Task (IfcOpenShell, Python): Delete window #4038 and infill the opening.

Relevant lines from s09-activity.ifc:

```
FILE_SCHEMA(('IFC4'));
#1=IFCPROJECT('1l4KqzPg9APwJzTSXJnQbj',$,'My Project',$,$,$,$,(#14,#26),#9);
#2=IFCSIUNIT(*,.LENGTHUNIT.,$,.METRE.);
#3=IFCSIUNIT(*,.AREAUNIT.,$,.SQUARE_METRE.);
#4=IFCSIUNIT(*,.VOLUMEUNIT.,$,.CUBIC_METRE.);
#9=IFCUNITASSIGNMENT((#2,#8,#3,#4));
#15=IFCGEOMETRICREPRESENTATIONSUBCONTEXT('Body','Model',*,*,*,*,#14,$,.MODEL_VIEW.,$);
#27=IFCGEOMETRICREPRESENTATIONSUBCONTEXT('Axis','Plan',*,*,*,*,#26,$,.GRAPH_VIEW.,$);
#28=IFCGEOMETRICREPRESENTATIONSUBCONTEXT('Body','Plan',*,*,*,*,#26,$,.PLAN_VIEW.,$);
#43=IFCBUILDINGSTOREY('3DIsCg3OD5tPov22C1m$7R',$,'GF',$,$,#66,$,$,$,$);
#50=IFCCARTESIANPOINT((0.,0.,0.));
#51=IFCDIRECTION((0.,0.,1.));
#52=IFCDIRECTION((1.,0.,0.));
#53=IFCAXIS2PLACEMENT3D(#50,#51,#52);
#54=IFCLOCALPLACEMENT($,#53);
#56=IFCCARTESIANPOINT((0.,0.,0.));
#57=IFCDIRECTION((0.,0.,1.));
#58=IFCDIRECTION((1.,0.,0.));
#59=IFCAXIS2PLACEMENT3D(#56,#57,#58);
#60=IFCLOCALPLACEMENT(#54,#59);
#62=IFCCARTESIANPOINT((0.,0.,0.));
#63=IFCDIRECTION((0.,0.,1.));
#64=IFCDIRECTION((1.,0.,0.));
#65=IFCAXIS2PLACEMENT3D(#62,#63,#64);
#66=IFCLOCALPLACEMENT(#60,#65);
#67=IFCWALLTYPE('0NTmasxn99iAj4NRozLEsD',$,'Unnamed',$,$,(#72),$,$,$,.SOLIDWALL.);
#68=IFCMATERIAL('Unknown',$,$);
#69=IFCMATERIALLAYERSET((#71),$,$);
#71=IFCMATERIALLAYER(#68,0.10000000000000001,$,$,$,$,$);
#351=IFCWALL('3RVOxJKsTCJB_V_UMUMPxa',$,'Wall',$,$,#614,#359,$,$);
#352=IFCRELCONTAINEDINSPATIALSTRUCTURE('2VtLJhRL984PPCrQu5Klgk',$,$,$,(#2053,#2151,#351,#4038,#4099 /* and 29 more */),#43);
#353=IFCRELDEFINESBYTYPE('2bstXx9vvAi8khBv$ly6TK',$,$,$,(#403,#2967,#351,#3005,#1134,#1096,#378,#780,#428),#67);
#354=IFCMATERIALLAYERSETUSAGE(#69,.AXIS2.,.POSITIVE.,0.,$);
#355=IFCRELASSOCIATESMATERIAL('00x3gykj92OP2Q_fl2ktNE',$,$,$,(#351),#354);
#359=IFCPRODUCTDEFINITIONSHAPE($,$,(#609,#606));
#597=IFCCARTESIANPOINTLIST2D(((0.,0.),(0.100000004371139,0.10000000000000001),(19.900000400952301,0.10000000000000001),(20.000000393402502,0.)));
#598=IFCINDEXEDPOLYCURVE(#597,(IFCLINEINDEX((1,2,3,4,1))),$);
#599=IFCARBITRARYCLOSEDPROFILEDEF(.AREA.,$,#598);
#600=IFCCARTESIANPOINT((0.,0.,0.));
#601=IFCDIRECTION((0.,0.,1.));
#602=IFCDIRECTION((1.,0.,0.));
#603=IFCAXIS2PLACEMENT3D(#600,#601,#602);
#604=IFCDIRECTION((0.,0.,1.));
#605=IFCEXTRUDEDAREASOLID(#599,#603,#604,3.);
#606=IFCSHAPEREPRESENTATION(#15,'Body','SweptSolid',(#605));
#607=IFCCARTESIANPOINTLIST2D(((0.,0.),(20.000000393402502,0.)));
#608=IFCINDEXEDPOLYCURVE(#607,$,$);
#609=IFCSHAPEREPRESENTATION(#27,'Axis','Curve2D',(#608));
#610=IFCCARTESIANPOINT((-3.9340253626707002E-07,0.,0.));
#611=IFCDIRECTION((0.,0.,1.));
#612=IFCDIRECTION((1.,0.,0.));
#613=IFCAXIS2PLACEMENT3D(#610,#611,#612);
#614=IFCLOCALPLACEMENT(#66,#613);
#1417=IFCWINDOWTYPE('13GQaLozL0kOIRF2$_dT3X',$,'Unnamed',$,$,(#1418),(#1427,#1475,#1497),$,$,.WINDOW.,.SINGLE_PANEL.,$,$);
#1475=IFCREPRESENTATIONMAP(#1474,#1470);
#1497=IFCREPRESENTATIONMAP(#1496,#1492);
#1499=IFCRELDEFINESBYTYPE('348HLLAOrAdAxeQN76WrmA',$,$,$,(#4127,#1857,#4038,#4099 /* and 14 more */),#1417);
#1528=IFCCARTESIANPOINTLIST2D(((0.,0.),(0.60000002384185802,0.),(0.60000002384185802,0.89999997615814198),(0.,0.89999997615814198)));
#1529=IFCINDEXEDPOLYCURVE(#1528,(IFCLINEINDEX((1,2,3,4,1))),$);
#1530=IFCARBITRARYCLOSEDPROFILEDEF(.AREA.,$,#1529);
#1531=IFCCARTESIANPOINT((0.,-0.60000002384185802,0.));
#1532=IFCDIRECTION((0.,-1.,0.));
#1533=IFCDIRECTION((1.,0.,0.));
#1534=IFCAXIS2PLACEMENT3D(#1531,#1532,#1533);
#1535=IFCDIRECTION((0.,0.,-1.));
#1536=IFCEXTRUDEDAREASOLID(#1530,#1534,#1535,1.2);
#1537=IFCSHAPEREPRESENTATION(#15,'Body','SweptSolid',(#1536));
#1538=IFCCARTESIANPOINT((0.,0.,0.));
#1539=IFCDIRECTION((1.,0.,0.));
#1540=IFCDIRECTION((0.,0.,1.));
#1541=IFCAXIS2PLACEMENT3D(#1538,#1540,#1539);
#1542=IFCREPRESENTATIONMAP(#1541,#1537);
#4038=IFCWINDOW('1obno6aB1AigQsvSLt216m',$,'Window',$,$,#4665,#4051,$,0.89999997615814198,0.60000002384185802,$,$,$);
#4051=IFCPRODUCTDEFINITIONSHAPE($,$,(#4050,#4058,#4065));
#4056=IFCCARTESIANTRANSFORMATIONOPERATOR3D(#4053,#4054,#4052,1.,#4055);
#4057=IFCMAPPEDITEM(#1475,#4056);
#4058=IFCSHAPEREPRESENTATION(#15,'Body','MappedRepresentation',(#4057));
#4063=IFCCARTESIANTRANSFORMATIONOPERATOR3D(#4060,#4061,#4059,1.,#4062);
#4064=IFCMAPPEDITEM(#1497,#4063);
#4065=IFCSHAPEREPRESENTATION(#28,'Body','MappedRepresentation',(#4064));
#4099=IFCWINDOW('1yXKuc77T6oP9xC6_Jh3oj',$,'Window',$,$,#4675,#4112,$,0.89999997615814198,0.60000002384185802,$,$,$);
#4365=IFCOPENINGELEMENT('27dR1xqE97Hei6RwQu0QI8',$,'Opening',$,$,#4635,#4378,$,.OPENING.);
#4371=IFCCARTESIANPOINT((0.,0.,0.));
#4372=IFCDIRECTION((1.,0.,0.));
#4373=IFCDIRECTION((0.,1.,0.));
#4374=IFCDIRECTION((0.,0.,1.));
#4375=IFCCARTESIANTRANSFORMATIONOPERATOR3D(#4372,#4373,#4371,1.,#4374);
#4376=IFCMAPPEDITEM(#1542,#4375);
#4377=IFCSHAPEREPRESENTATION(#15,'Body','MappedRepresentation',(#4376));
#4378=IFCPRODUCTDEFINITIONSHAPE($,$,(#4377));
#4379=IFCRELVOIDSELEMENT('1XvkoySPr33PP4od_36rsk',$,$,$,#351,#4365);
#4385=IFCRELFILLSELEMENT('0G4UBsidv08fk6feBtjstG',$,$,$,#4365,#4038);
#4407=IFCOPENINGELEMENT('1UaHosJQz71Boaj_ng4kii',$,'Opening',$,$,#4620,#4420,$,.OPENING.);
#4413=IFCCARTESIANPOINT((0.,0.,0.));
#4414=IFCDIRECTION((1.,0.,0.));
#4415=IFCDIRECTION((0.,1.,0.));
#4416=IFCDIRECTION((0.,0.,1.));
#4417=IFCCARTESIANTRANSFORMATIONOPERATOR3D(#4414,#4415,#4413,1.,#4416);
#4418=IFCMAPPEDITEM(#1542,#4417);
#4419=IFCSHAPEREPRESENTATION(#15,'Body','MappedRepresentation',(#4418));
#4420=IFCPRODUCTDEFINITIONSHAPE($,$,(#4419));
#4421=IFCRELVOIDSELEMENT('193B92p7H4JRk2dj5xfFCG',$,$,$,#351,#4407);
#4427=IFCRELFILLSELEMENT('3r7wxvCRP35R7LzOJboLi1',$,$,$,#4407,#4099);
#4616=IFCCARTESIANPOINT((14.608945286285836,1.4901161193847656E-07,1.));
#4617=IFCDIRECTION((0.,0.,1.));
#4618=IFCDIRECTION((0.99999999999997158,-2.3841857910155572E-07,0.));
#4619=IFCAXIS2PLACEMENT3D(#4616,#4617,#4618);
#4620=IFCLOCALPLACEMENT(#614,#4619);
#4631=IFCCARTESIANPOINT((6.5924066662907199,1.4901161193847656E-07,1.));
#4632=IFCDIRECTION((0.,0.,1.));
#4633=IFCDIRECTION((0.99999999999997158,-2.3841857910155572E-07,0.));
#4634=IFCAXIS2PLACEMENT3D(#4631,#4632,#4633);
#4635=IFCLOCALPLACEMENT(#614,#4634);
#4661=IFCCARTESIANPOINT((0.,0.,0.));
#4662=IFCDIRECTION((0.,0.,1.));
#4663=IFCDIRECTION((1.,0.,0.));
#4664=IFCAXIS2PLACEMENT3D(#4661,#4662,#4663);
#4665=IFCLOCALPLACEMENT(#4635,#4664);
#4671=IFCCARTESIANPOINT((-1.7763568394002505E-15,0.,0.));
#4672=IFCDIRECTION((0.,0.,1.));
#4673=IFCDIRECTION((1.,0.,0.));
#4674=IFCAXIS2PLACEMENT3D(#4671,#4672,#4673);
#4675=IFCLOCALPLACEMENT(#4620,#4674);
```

```python
import ifcopenshell
import ifcopenshell.api.feature
import ifcopenshell.api.root
import ifcopenshell.geom
import ifcopenshell.util.shape

model = ifcopenshell.open("s09-activity.ifc")
settings = ifcopenshell.geom.settings()


def volume(element):
    """Net volume in cubic metres, openings subtracted."""
    shape = ifcopenshell.geom.create_shape(settings, element)
    return ifcopenshell.util.shape.get_volume(shape.geometry)


window = model.by_guid("1obno6aB1AigQsvSLt216m")
opening = window.FillsVoids[0].RelatingOpeningElement
wall = opening.VoidsElements[0].RelatingBuildingElement
before = volume(wall)

ifcopenshell.api.root.remove_product(model, product=window)
ifcopenshell.api.feature.remove_feature(model, feature=opening)

after = volume(wall)

print(f"wall volume {before:.3f} -> {after:.3f} m3")

model.write("s09-activity_rev.ifc")
```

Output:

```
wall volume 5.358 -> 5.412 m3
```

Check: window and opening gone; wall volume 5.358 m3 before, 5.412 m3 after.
